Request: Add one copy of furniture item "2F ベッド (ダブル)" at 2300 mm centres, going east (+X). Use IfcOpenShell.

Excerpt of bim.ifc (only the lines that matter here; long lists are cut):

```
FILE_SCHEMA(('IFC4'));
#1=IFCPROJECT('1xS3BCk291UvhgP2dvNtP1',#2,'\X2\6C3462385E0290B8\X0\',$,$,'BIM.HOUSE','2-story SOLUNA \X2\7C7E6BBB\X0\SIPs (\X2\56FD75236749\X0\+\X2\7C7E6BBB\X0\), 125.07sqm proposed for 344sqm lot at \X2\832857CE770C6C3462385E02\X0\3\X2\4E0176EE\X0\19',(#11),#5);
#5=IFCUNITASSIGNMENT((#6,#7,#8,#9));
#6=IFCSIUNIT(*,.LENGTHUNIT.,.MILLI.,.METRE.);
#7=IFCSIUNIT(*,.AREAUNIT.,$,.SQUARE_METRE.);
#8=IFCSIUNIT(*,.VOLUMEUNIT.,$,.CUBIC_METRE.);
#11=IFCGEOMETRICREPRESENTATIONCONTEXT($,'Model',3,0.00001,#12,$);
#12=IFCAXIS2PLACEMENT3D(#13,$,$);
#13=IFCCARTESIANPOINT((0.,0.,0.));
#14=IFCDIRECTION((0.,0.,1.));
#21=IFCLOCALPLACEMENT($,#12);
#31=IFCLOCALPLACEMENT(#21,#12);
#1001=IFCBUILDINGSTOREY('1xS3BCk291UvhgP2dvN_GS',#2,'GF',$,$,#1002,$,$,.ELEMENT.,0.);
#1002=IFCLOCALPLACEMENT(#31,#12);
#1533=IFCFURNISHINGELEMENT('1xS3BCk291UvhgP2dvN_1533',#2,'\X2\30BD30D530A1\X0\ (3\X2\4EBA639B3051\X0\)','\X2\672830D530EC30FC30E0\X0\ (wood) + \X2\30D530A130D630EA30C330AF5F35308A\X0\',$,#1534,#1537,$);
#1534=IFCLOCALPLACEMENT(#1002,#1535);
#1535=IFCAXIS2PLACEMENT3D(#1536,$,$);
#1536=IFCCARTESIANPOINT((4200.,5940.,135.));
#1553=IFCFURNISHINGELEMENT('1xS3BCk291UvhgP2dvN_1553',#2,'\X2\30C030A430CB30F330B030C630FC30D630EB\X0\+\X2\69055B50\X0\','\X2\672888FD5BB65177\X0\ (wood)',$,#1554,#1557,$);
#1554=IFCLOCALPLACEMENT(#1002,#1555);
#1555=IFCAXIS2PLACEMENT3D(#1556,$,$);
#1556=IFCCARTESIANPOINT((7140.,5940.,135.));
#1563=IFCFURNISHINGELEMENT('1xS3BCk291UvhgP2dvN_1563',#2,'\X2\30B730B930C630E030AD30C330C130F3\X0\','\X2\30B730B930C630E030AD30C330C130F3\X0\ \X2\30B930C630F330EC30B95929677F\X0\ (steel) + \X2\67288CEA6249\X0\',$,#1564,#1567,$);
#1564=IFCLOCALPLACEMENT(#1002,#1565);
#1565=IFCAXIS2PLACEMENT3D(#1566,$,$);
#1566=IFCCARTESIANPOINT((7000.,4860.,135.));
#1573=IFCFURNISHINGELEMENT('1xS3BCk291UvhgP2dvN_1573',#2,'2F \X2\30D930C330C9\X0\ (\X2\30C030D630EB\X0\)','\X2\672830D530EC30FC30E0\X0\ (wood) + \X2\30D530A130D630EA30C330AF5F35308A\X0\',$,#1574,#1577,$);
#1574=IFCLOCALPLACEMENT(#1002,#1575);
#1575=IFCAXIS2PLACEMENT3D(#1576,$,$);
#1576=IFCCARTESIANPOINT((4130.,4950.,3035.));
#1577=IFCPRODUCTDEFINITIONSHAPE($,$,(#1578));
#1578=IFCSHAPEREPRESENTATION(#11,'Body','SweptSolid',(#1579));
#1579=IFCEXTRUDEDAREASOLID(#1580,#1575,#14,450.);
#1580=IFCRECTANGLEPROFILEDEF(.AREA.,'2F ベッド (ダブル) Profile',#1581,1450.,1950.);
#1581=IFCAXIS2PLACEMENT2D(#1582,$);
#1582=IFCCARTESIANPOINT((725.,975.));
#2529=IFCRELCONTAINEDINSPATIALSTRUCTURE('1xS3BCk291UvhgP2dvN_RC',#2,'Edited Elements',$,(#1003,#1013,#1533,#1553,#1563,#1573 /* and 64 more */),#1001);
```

```python
import numpy as np
import ifcopenshell
import ifcopenshell.api.geometry
import ifcopenshell.api.root
import ifcopenshell.util.element
import ifcopenshell.util.placement
import ifcopenshell.util.unit

model = ifcopenshell.open("bim.ifc")
unit_scale = ifcopenshell.util.unit.calculate_unit_scale(model)


def reuse_history(source, copy):
    """copy_class also copies each property set's owner history, people and application; keep the originals."""
    for rel in copy.IsDefinedBy:
        if rel.is_a("IfcRelDefinesByProperties") and (history := rel.RelatingPropertyDefinition.OwnerHistory):
            rel.RelatingPropertyDefinition.OwnerHistory = source.OwnerHistory
            ifcopenshell.util.element.remove_deep2(model, history)


source = model.by_guid("1xS3BCk291UvhgP2dvN_1573")
base = ifcopenshell.util.placement.get_local_placement(source.ObjectPlacement)
step = np.array([1.0, 0.0, 0.0]) * 2.3 / unit_scale

for i in range(1, 2):
    copy = ifcopenshell.api.root.copy_class(model, product=source)
    copy.Representation = ifcopenshell.util.element.copy_deep(
        model, source.Representation, exclude=["IfcGeometricRepresentationContext", "IfcRepresentationMap"]
    )
    reuse_history(source, copy)
    matrix = base.copy()
    matrix[:3, 3] += i * step
    print("added at", matrix[:3, 3].round(3) + 0.0)
    ifcopenshell.api.geometry.edit_object_placement(model, product=copy, matrix=matrix, is_si=False)

model.write("bim_rev.ifc")
```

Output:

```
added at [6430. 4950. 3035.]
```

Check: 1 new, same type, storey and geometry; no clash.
